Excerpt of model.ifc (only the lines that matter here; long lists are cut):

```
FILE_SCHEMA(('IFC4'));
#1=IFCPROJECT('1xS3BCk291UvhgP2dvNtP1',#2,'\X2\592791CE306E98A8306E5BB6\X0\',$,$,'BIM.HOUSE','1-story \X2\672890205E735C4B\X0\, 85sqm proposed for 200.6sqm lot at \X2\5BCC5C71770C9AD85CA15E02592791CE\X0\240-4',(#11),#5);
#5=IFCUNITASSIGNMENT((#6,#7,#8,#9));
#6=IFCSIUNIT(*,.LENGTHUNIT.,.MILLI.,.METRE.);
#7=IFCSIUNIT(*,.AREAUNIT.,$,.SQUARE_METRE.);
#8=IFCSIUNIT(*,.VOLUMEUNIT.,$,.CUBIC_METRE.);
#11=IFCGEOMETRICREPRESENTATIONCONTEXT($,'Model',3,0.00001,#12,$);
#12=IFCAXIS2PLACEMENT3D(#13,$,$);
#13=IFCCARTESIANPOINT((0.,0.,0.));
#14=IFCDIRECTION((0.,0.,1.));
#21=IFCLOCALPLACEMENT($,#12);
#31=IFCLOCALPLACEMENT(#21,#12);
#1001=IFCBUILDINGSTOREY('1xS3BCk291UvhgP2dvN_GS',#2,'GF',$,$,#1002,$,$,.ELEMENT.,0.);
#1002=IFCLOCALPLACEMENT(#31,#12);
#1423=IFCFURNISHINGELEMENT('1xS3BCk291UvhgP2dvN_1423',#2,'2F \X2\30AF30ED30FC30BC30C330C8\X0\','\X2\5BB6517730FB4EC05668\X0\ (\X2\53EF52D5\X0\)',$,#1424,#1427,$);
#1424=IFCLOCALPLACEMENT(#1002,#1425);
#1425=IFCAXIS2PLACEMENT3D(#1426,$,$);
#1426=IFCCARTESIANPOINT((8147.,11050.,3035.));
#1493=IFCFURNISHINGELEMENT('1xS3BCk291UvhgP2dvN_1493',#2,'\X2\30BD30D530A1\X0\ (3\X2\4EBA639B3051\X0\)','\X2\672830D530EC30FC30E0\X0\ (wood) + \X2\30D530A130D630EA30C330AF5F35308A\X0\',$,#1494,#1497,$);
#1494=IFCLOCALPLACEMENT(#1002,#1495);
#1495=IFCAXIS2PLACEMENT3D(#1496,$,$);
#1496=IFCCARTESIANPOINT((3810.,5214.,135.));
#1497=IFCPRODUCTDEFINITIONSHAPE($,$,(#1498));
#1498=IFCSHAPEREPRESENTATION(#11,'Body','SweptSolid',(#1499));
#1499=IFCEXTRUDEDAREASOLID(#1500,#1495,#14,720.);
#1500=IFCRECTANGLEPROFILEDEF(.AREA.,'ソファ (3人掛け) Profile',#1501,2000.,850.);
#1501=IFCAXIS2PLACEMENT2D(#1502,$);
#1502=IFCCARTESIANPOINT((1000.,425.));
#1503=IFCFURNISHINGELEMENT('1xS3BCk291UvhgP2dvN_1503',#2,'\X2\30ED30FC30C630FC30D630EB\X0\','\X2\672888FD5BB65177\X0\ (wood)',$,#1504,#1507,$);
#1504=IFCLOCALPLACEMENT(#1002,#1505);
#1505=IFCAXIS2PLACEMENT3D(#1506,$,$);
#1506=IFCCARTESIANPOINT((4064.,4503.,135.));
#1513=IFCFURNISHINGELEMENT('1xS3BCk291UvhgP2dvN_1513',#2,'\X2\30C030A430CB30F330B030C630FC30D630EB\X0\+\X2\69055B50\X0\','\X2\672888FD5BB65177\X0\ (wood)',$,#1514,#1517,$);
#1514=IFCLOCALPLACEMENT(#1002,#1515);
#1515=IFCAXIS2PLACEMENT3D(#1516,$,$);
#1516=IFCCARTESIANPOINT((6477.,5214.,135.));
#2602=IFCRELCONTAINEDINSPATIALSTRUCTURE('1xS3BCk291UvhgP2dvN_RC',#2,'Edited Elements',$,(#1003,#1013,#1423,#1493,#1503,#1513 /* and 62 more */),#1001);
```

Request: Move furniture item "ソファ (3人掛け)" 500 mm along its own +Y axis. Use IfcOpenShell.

```python
import ifcopenshell
import ifcopenshell.api.geometry
import ifcopenshell.util.placement

model = ifcopenshell.open("model.ifc")

item = model.by_guid("1xS3BCk291UvhgP2dvN_1493")
matrix = ifcopenshell.util.placement.get_local_placement(item.ObjectPlacement)
matrix[:3, 3] += matrix[:3, 1] * 500.0
ifcopenshell.api.geometry.edit_object_placement(model, product=item, matrix=matrix, is_si=False)

print(ifcopenshell.util.placement.get_local_placement(item.ObjectPlacement).round(3) + 0.0)

model.write("model-out.ifc")
```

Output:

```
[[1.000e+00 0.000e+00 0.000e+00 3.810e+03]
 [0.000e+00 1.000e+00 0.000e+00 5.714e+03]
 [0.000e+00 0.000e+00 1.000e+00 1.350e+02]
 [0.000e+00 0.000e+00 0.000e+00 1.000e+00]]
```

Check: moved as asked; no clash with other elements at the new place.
